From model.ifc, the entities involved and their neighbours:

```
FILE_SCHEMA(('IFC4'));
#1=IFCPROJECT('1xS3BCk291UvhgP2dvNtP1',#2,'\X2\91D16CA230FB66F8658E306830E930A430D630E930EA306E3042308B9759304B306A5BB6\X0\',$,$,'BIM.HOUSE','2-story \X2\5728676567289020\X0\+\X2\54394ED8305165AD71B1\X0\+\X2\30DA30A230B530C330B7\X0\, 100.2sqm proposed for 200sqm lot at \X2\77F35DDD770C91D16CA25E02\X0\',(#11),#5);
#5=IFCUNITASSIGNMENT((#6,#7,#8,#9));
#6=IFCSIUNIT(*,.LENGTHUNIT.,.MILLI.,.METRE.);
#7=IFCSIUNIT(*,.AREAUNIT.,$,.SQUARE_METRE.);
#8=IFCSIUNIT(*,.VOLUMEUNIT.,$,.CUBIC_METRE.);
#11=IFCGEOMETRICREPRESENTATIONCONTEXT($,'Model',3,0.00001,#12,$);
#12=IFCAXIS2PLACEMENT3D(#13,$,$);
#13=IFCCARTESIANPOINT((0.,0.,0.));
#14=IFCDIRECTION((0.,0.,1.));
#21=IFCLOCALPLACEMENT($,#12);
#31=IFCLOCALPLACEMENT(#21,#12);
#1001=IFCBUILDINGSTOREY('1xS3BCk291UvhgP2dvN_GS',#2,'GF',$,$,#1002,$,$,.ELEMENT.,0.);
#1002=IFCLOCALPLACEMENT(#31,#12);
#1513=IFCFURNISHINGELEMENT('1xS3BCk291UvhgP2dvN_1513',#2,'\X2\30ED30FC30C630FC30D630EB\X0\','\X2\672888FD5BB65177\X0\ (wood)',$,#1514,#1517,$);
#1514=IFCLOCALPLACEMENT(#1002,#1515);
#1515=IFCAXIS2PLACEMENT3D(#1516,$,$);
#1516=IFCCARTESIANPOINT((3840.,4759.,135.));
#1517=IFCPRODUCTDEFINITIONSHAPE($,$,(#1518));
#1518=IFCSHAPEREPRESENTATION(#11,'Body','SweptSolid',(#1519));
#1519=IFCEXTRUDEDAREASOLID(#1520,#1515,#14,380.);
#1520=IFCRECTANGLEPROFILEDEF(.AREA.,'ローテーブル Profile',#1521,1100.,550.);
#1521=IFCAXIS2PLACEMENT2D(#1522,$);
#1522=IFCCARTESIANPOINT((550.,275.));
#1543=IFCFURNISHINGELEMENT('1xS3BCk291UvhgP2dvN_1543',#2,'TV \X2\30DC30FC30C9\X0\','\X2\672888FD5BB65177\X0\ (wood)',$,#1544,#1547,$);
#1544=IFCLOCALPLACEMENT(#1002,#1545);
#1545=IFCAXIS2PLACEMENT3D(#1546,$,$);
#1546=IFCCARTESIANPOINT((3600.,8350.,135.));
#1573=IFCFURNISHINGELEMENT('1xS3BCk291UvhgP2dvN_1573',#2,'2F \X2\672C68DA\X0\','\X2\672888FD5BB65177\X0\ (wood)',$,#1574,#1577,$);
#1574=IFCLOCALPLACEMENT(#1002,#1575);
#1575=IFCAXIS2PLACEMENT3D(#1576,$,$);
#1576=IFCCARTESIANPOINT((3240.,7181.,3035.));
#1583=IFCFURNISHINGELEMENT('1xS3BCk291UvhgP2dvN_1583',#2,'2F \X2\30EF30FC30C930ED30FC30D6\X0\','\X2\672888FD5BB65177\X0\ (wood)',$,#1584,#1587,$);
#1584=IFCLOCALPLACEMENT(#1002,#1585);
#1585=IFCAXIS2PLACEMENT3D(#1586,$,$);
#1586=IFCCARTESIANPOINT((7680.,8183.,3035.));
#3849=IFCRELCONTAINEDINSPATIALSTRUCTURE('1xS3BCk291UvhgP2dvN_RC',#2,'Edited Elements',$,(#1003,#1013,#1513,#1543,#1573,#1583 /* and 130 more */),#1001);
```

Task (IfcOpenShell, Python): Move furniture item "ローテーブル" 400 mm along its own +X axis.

```python
import ifcopenshell
import ifcopenshell.api.geometry
import ifcopenshell.util.placement
import ifcopenshell.util.unit

model = ifcopenshell.open("model.ifc")
unit_scale = ifcopenshell.util.unit.calculate_unit_scale(model)

item = model.by_guid("1xS3BCk291UvhgP2dvN_1513")
matrix = ifcopenshell.util.placement.get_local_placement(item.ObjectPlacement)
matrix[:3, 3] += matrix[:3, 0] * 0.4 / unit_scale
ifcopenshell.api.geometry.edit_object_placement(model, product=item, matrix=matrix, is_si=False)

print(ifcopenshell.util.placement.get_local_placement(item.ObjectPlacement).round(3) + 0.0)

model.write("model-out.ifc")
```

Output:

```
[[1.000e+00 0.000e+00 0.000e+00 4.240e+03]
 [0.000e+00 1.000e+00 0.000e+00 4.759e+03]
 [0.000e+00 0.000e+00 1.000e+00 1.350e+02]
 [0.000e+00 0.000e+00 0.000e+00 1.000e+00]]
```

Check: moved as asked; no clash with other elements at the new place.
